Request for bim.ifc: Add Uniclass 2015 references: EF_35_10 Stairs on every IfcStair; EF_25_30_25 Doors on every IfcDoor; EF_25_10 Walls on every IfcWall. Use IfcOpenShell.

First a look at what the model holds.

```python
import ifcopenshell

model = ifcopenshell.open("bim.ifc")
print(model.schema)
print("classifications:", [c.Name for c in model.by_type("IfcClassification")])
for ifc_class in ("IfcDoor", "IfcRoof", "IfcStair", "IfcWall", "IfcWindow"):
    print(ifc_class, len(model.by_type(ifc_class)))
```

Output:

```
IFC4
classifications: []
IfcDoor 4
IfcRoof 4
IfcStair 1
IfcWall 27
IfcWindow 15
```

```python
import ifcopenshell
import ifcopenshell.api.classification

model = ifcopenshell.open("bim.ifc")

system = ifcopenshell.api.classification.add_classification(model, classification="Uniclass 2015")

codes = {
    "IfcStair": ("EF_35_10", "Stairs"),
    "IfcDoor": ("EF_25_30_25", "Doors"),
    "IfcWall": ("EF_25_10", "Walls"),
}
for ifc_class, (code, name) in codes.items():
    products = model.by_type(ifc_class)
    ifcopenshell.api.classification.add_reference(
        model, products=products, classification=system, identification=code, name=name
    )
    print(code, len(products))

model.write("bim_v2.ifc")
```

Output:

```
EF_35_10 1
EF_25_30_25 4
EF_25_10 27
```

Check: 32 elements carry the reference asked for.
